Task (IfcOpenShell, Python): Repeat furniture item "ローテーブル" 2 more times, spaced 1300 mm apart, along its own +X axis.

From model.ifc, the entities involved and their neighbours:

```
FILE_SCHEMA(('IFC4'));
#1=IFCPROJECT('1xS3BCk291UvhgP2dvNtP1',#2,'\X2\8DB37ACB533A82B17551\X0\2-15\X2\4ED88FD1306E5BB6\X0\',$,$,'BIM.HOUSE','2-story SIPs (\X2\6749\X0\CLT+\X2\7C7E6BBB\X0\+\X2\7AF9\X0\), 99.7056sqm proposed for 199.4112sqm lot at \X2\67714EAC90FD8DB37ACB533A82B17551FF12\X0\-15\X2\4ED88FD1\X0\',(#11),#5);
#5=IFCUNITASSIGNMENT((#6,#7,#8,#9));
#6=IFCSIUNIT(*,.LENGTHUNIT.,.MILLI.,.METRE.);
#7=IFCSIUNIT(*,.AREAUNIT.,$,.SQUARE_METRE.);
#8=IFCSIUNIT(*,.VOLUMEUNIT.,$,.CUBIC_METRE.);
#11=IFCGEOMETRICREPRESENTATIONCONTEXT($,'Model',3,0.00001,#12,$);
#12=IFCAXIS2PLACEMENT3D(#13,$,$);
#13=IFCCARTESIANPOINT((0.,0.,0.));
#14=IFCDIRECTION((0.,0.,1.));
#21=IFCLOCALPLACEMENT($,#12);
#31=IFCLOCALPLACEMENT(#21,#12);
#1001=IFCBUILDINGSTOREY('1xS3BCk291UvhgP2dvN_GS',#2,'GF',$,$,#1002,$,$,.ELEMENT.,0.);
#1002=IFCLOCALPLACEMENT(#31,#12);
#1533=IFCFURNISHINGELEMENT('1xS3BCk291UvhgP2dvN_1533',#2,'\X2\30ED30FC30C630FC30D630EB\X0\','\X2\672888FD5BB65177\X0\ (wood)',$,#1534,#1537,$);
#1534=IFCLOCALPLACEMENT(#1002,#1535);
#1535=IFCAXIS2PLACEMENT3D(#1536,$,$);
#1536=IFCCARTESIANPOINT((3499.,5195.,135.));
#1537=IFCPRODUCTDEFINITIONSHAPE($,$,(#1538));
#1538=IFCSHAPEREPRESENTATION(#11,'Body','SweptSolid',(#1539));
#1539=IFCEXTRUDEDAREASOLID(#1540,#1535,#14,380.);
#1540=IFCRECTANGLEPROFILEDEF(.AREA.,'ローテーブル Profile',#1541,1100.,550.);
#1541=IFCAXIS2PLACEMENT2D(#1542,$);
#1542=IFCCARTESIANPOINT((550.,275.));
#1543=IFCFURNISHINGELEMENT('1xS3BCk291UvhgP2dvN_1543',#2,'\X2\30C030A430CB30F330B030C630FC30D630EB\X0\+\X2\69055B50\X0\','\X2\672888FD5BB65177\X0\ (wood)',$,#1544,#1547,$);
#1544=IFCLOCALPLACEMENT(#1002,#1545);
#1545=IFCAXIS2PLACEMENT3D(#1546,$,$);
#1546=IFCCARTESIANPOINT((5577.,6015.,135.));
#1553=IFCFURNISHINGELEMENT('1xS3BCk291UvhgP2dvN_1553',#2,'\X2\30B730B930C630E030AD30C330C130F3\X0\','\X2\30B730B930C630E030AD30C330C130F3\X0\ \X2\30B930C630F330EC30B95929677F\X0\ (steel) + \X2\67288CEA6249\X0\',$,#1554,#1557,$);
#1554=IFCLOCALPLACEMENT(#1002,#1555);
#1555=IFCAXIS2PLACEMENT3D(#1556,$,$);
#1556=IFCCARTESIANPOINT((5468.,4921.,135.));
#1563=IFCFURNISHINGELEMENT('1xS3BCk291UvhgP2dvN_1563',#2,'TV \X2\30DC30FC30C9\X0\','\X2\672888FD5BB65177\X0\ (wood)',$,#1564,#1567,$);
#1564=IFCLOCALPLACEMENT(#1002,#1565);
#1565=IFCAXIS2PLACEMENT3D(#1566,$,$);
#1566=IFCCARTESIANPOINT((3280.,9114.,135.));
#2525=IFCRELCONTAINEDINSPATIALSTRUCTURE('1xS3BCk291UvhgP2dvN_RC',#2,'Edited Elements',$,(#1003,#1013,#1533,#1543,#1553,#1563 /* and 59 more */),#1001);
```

```python
import ifcopenshell
import ifcopenshell.api.geometry
import ifcopenshell.api.root
import ifcopenshell.util.element
import ifcopenshell.util.placement

model = ifcopenshell.open("model.ifc")


def reuse_history(source, copy):
    """copy_class also copies each property set's owner history, people and application; keep the originals."""
    for rel in copy.IsDefinedBy:
        if rel.is_a("IfcRelDefinesByProperties") and (history := rel.RelatingPropertyDefinition.OwnerHistory):
            rel.RelatingPropertyDefinition.OwnerHistory = source.OwnerHistory
            ifcopenshell.util.element.remove_deep2(model, history)


source = model.by_guid("1xS3BCk291UvhgP2dvN_1533")
base = ifcopenshell.util.placement.get_local_placement(source.ObjectPlacement)
step = base[:3, 0] * 1300.0

for i in range(1, 3):
    copy = ifcopenshell.api.root.copy_class(model, product=source)
    copy.Representation = ifcopenshell.util.element.copy_deep(
        model, source.Representation, exclude=["IfcGeometricRepresentationContext", "IfcRepresentationMap"]
    )
    reuse_history(source, copy)
    matrix = base.copy()
    matrix[:3, 3] += i * step
    print("added at", matrix[:3, 3].round(3) + 0.0)
    ifcopenshell.api.geometry.edit_object_placement(model, product=copy, matrix=matrix, is_si=False)

model.write("model_updated.ifc")
```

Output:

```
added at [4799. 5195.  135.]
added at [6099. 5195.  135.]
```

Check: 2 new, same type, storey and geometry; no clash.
